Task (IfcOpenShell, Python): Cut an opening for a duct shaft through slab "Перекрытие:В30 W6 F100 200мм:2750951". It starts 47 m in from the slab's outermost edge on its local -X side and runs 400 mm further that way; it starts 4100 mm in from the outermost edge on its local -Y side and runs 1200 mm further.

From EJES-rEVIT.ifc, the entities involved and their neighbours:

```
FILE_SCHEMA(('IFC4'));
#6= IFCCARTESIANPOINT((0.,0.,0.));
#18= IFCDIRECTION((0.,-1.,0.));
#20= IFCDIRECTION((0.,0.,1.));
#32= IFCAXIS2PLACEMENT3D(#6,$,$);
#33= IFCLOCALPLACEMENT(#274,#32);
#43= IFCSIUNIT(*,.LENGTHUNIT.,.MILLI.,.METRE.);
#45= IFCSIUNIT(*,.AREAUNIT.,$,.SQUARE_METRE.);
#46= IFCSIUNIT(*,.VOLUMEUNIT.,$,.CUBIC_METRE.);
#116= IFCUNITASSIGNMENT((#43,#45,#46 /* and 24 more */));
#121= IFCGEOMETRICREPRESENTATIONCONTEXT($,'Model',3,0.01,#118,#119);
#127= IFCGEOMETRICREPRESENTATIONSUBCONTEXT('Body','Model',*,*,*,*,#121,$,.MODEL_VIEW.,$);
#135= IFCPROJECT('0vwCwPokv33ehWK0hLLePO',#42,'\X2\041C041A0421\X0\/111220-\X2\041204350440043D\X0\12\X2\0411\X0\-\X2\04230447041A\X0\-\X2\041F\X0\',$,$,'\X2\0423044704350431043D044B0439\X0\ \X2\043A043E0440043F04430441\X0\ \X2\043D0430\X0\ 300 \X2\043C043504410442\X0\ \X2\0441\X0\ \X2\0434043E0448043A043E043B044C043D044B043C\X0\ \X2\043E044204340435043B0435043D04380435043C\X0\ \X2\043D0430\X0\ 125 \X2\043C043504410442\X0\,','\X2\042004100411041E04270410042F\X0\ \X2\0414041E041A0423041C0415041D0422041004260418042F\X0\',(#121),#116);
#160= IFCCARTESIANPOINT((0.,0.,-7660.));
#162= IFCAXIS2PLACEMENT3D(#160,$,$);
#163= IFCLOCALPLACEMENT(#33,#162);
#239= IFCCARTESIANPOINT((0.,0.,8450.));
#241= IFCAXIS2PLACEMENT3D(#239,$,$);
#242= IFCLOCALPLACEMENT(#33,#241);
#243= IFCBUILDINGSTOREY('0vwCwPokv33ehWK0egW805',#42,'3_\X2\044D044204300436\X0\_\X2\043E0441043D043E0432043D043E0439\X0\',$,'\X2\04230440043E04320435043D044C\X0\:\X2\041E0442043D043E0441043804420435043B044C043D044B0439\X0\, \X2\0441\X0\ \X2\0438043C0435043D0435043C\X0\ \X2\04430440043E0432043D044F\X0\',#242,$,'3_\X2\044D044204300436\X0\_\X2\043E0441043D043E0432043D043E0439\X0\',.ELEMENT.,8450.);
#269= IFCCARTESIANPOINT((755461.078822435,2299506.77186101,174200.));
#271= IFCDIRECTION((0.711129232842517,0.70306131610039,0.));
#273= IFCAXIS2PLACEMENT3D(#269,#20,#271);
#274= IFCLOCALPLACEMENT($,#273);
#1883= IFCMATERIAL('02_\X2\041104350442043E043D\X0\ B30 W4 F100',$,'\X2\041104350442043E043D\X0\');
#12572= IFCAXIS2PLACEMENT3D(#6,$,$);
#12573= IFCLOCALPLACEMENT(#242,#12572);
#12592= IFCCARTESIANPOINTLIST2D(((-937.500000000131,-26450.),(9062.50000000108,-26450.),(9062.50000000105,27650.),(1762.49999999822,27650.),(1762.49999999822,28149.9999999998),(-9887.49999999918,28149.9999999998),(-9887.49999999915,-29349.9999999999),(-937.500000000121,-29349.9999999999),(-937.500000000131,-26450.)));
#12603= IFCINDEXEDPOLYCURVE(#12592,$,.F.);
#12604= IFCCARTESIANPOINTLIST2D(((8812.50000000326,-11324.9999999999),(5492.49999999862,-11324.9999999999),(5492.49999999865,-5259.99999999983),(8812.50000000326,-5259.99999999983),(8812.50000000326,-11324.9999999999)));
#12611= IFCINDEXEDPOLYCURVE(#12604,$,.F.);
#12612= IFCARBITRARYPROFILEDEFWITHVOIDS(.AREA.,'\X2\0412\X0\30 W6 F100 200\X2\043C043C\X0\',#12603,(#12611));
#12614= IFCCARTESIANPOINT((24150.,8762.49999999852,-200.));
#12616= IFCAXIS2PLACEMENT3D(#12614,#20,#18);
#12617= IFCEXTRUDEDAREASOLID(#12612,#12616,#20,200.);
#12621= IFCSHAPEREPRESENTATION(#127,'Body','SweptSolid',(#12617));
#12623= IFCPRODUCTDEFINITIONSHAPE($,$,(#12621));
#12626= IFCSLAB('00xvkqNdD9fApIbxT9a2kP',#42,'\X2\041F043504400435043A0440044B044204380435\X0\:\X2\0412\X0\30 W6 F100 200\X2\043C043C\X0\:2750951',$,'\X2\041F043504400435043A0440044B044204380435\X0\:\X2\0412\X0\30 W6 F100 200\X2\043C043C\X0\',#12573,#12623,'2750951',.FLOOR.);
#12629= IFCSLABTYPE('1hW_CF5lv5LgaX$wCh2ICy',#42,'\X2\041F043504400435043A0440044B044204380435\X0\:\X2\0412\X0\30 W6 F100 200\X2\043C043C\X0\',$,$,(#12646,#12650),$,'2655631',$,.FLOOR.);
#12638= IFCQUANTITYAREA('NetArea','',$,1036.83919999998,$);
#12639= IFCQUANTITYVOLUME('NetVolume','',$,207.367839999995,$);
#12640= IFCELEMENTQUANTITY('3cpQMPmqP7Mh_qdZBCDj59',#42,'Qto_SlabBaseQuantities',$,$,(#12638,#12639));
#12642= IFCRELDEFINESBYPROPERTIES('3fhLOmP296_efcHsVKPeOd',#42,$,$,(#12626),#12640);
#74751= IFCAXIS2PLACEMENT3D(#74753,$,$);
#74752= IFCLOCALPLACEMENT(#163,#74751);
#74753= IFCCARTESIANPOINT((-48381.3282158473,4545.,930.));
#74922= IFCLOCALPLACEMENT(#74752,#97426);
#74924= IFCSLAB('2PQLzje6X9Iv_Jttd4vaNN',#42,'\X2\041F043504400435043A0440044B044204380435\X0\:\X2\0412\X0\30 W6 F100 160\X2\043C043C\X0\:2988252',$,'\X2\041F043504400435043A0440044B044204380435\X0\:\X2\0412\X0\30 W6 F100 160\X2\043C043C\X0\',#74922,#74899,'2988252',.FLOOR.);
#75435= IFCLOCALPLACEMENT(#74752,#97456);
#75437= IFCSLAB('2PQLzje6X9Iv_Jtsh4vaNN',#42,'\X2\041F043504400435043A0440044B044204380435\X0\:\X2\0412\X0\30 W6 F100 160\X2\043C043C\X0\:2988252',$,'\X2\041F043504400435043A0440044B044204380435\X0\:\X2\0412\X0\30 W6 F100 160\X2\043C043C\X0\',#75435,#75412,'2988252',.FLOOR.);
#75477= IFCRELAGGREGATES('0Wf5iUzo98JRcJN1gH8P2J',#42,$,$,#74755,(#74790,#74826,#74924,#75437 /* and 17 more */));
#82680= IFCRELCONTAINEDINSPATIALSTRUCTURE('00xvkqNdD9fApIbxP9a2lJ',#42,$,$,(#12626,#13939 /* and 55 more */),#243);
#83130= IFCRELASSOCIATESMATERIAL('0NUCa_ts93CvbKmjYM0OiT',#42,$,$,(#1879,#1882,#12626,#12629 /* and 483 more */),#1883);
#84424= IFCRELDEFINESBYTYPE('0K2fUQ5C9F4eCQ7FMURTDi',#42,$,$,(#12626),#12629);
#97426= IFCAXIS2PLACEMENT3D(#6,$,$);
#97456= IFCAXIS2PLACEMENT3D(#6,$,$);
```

```python
import numpy as np
import ifcopenshell
import ifcopenshell.api.feature
import ifcopenshell.api.geometry
import ifcopenshell.api.pset
import ifcopenshell.api.root
import ifcopenshell.geom
import ifcopenshell.util.element
import ifcopenshell.util.placement
import ifcopenshell.util.representation
import ifcopenshell.util.shape
import ifcopenshell.util.unit

model = ifcopenshell.open("EJES-rEVIT.ifc")
unit_scale = ifcopenshell.util.unit.calculate_unit_scale(model)
area_scale = ifcopenshell.util.unit.calculate_unit_scale(model, "AREAUNIT")
volume_scale = ifcopenshell.util.unit.calculate_unit_scale(model, "VOLUMEUNIT")
settings = ifcopenshell.geom.settings()


def volume(element):
    """Net volume in cubic metres, openings subtracted."""
    shape = ifcopenshell.geom.create_shape(settings, element)
    return ifcopenshell.util.shape.get_volume(shape.geometry)


slab = model.by_guid("00xvkqNdD9fApIbxT9a2kP")
before = volume(slab)

# Extent in the slab's own axes, in metres. The edges named are its -X and -Y sides.
slab_shape = ifcopenshell.geom.create_shape(settings, slab)
vertices = ifcopenshell.util.shape.get_vertices(slab_shape.geometry)
x_min, y_min, bottom = vertices.min(axis=0)
top = vertices[:, 2].max()

opening = ifcopenshell.api.root.create_entity(model, ifc_class="IfcOpeningElement", name="Duct shaft opening", predefined_type="OPENING")
context = ifcopenshell.util.representation.get_context(model, "Model", "Body", "MODEL_VIEW")
width, depth = 0.4, 1.2
outline = [(0.0, 0.0), (width, 0.0), (width, depth), (0.0, depth), (0.0, 0.0)]
# Overshoot both faces by 50 mm so the cut is clean.
shape = ifcopenshell.api.geometry.add_slab_representation(
    model, context=context, depth=top - bottom + 0.1, polyline=outline
)
ifcopenshell.api.geometry.assign_representation(model, product=opening, representation=shape)

matrix = ifcopenshell.util.placement.get_local_placement(slab.ObjectPlacement)
matrix[:, 3] = matrix @ np.append(np.array([x_min + 47, y_min + 4.1, bottom - 0.05]) / unit_scale, 1.0)
ifcopenshell.api.geometry.edit_object_placement(model, product=opening, matrix=matrix, is_si=False)
ifcopenshell.api.feature.add_feature(model, feature=opening, element=slab)

after = volume(slab)

# Update the slab's stored quantities.
qto = model.by_id(ifcopenshell.util.element.get_pset(slab, "Qto_SlabBaseQuantities", should_inherit=False)["id"])
ifcopenshell.api.pset.edit_qto(model, qto=qto, properties={
    "NetArea": after / (top - bottom) / area_scale,
    "NetVolume": after / volume_scale,
})

print(f"slab volume {before:.3f} -> {after:.3f} m3")

model.write("EJES-rEVIT_edited.ifc")
```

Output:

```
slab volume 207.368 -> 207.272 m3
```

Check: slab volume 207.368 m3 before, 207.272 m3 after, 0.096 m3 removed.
